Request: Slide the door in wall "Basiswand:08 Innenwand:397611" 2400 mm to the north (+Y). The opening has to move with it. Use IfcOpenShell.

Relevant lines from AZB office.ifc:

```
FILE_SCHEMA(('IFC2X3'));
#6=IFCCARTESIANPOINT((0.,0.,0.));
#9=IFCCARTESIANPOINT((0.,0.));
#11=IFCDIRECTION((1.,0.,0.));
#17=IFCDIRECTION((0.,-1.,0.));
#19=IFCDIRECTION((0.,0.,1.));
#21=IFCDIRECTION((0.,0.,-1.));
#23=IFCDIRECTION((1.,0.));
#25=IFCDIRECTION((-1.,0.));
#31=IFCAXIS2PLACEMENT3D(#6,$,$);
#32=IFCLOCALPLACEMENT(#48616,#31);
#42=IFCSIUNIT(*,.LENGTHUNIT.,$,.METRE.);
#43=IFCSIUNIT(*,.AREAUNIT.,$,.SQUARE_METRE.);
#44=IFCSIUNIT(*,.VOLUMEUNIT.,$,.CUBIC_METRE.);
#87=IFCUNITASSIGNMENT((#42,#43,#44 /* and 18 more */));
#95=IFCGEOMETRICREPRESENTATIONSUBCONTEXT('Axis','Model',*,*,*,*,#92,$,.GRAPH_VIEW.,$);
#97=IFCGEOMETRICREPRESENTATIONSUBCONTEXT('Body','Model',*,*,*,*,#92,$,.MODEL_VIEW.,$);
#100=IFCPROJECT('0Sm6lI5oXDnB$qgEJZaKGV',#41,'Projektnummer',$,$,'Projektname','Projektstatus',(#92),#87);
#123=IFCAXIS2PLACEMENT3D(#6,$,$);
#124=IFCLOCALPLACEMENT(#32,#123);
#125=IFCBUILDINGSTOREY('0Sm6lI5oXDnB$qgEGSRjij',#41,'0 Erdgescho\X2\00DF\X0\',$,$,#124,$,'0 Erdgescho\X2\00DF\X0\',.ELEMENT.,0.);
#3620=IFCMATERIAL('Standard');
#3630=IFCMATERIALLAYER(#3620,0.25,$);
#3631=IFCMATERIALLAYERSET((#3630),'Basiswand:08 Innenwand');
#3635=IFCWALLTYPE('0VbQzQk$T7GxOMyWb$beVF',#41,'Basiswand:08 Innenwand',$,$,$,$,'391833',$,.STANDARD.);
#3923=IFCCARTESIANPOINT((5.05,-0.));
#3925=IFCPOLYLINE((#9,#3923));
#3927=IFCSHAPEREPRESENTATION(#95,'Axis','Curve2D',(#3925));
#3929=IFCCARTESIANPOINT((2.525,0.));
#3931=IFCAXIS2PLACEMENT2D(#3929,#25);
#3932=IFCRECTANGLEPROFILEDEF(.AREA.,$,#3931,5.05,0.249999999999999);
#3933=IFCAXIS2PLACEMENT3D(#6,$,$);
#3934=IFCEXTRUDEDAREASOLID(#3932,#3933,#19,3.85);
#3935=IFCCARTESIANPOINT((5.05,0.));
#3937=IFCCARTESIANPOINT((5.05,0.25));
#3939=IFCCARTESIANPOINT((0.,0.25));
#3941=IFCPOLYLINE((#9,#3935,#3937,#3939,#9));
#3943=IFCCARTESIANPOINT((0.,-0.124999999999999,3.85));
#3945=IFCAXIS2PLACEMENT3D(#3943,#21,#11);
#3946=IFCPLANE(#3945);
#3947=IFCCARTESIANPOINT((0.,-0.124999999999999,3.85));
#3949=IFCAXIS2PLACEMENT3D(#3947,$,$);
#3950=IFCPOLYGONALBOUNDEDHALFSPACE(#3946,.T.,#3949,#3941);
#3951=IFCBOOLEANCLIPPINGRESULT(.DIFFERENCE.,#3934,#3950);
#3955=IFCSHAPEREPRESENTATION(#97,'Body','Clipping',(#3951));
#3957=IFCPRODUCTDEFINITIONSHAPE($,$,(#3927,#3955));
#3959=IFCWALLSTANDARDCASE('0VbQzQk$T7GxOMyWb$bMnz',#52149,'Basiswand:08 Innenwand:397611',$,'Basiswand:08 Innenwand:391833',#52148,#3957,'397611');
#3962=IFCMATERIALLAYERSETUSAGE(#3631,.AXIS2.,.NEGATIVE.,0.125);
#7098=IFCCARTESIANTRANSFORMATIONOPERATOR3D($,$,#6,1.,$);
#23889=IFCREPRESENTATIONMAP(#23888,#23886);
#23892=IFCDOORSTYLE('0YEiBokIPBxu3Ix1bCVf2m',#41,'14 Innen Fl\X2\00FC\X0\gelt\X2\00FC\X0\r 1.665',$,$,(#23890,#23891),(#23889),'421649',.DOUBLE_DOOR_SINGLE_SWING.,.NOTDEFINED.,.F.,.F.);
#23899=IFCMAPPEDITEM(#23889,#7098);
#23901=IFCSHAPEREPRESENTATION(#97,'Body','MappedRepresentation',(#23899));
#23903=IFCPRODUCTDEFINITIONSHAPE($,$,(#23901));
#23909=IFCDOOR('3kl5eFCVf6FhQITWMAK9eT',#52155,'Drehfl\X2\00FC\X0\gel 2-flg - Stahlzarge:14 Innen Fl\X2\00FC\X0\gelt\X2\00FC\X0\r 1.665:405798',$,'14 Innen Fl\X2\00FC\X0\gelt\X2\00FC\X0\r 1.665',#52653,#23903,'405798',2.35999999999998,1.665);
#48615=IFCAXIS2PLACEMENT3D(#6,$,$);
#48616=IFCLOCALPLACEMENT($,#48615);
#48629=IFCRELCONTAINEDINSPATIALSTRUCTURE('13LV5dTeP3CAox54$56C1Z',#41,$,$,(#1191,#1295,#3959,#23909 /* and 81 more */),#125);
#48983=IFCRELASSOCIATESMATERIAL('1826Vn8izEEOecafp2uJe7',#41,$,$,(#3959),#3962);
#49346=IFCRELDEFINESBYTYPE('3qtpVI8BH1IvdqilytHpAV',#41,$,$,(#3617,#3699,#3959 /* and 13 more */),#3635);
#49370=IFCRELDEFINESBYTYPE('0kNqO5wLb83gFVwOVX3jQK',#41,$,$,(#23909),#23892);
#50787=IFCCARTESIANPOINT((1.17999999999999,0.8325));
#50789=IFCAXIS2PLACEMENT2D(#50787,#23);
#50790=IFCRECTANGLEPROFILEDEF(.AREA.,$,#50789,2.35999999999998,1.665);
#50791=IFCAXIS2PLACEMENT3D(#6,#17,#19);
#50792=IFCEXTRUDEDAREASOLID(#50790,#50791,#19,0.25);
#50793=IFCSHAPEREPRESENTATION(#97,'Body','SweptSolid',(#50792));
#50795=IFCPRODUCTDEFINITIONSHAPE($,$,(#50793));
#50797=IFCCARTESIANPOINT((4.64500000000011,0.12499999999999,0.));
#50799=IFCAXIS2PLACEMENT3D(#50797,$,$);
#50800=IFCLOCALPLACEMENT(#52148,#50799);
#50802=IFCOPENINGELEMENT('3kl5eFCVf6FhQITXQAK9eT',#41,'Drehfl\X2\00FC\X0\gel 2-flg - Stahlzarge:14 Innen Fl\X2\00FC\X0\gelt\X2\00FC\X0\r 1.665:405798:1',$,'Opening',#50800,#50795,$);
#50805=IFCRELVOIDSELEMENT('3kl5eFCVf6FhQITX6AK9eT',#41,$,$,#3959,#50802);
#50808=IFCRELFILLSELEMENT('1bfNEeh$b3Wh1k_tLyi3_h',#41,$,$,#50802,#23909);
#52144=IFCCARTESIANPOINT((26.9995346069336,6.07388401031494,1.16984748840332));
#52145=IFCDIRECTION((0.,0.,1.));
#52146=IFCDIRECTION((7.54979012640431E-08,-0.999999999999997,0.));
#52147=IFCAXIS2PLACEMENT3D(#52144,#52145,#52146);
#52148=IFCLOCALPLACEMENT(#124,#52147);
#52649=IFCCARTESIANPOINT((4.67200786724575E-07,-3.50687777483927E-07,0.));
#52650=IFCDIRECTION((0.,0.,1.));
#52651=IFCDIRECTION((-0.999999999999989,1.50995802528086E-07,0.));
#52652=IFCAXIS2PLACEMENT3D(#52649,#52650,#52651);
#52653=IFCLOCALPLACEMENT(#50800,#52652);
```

```python
import ifcopenshell
import ifcopenshell.api.geometry
import ifcopenshell.util.placement
import ifcopenshell.util.unit

model = ifcopenshell.open("AZB office.ifc")
unit_scale = ifcopenshell.util.unit.calculate_unit_scale(model)

door = model.by_guid("3kl5eFCVf6FhQITWMAK9eT")
opening = door.FillsVoids[0].RelatingOpeningElement
wall = opening.VoidsElements[0].RelatingBuildingElement

wall_matrix = ifcopenshell.util.placement.get_local_placement(wall.ObjectPlacement)
shift = wall_matrix[:3, 0] * -2.4 / unit_scale
before = ifcopenshell.util.placement.get_local_placement(door.ObjectPlacement)[:3, 3].copy()

# The door is placed relative to its opening, so it follows when the opening moves.
matrix = ifcopenshell.util.placement.get_local_placement(opening.ObjectPlacement)
matrix[:3, 3] += shift
ifcopenshell.api.geometry.edit_object_placement(
    model, product=opening, matrix=matrix, is_si=False, should_transform_children=True
)

after = ifcopenshell.util.placement.get_local_placement(door.ObjectPlacement)[:3, 3]
print("door moved by", (after - before).round(3) + 0.0)

model.write("AZB office_edited.ifc")
```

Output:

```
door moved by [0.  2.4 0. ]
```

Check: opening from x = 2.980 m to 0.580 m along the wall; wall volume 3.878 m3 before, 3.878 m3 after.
